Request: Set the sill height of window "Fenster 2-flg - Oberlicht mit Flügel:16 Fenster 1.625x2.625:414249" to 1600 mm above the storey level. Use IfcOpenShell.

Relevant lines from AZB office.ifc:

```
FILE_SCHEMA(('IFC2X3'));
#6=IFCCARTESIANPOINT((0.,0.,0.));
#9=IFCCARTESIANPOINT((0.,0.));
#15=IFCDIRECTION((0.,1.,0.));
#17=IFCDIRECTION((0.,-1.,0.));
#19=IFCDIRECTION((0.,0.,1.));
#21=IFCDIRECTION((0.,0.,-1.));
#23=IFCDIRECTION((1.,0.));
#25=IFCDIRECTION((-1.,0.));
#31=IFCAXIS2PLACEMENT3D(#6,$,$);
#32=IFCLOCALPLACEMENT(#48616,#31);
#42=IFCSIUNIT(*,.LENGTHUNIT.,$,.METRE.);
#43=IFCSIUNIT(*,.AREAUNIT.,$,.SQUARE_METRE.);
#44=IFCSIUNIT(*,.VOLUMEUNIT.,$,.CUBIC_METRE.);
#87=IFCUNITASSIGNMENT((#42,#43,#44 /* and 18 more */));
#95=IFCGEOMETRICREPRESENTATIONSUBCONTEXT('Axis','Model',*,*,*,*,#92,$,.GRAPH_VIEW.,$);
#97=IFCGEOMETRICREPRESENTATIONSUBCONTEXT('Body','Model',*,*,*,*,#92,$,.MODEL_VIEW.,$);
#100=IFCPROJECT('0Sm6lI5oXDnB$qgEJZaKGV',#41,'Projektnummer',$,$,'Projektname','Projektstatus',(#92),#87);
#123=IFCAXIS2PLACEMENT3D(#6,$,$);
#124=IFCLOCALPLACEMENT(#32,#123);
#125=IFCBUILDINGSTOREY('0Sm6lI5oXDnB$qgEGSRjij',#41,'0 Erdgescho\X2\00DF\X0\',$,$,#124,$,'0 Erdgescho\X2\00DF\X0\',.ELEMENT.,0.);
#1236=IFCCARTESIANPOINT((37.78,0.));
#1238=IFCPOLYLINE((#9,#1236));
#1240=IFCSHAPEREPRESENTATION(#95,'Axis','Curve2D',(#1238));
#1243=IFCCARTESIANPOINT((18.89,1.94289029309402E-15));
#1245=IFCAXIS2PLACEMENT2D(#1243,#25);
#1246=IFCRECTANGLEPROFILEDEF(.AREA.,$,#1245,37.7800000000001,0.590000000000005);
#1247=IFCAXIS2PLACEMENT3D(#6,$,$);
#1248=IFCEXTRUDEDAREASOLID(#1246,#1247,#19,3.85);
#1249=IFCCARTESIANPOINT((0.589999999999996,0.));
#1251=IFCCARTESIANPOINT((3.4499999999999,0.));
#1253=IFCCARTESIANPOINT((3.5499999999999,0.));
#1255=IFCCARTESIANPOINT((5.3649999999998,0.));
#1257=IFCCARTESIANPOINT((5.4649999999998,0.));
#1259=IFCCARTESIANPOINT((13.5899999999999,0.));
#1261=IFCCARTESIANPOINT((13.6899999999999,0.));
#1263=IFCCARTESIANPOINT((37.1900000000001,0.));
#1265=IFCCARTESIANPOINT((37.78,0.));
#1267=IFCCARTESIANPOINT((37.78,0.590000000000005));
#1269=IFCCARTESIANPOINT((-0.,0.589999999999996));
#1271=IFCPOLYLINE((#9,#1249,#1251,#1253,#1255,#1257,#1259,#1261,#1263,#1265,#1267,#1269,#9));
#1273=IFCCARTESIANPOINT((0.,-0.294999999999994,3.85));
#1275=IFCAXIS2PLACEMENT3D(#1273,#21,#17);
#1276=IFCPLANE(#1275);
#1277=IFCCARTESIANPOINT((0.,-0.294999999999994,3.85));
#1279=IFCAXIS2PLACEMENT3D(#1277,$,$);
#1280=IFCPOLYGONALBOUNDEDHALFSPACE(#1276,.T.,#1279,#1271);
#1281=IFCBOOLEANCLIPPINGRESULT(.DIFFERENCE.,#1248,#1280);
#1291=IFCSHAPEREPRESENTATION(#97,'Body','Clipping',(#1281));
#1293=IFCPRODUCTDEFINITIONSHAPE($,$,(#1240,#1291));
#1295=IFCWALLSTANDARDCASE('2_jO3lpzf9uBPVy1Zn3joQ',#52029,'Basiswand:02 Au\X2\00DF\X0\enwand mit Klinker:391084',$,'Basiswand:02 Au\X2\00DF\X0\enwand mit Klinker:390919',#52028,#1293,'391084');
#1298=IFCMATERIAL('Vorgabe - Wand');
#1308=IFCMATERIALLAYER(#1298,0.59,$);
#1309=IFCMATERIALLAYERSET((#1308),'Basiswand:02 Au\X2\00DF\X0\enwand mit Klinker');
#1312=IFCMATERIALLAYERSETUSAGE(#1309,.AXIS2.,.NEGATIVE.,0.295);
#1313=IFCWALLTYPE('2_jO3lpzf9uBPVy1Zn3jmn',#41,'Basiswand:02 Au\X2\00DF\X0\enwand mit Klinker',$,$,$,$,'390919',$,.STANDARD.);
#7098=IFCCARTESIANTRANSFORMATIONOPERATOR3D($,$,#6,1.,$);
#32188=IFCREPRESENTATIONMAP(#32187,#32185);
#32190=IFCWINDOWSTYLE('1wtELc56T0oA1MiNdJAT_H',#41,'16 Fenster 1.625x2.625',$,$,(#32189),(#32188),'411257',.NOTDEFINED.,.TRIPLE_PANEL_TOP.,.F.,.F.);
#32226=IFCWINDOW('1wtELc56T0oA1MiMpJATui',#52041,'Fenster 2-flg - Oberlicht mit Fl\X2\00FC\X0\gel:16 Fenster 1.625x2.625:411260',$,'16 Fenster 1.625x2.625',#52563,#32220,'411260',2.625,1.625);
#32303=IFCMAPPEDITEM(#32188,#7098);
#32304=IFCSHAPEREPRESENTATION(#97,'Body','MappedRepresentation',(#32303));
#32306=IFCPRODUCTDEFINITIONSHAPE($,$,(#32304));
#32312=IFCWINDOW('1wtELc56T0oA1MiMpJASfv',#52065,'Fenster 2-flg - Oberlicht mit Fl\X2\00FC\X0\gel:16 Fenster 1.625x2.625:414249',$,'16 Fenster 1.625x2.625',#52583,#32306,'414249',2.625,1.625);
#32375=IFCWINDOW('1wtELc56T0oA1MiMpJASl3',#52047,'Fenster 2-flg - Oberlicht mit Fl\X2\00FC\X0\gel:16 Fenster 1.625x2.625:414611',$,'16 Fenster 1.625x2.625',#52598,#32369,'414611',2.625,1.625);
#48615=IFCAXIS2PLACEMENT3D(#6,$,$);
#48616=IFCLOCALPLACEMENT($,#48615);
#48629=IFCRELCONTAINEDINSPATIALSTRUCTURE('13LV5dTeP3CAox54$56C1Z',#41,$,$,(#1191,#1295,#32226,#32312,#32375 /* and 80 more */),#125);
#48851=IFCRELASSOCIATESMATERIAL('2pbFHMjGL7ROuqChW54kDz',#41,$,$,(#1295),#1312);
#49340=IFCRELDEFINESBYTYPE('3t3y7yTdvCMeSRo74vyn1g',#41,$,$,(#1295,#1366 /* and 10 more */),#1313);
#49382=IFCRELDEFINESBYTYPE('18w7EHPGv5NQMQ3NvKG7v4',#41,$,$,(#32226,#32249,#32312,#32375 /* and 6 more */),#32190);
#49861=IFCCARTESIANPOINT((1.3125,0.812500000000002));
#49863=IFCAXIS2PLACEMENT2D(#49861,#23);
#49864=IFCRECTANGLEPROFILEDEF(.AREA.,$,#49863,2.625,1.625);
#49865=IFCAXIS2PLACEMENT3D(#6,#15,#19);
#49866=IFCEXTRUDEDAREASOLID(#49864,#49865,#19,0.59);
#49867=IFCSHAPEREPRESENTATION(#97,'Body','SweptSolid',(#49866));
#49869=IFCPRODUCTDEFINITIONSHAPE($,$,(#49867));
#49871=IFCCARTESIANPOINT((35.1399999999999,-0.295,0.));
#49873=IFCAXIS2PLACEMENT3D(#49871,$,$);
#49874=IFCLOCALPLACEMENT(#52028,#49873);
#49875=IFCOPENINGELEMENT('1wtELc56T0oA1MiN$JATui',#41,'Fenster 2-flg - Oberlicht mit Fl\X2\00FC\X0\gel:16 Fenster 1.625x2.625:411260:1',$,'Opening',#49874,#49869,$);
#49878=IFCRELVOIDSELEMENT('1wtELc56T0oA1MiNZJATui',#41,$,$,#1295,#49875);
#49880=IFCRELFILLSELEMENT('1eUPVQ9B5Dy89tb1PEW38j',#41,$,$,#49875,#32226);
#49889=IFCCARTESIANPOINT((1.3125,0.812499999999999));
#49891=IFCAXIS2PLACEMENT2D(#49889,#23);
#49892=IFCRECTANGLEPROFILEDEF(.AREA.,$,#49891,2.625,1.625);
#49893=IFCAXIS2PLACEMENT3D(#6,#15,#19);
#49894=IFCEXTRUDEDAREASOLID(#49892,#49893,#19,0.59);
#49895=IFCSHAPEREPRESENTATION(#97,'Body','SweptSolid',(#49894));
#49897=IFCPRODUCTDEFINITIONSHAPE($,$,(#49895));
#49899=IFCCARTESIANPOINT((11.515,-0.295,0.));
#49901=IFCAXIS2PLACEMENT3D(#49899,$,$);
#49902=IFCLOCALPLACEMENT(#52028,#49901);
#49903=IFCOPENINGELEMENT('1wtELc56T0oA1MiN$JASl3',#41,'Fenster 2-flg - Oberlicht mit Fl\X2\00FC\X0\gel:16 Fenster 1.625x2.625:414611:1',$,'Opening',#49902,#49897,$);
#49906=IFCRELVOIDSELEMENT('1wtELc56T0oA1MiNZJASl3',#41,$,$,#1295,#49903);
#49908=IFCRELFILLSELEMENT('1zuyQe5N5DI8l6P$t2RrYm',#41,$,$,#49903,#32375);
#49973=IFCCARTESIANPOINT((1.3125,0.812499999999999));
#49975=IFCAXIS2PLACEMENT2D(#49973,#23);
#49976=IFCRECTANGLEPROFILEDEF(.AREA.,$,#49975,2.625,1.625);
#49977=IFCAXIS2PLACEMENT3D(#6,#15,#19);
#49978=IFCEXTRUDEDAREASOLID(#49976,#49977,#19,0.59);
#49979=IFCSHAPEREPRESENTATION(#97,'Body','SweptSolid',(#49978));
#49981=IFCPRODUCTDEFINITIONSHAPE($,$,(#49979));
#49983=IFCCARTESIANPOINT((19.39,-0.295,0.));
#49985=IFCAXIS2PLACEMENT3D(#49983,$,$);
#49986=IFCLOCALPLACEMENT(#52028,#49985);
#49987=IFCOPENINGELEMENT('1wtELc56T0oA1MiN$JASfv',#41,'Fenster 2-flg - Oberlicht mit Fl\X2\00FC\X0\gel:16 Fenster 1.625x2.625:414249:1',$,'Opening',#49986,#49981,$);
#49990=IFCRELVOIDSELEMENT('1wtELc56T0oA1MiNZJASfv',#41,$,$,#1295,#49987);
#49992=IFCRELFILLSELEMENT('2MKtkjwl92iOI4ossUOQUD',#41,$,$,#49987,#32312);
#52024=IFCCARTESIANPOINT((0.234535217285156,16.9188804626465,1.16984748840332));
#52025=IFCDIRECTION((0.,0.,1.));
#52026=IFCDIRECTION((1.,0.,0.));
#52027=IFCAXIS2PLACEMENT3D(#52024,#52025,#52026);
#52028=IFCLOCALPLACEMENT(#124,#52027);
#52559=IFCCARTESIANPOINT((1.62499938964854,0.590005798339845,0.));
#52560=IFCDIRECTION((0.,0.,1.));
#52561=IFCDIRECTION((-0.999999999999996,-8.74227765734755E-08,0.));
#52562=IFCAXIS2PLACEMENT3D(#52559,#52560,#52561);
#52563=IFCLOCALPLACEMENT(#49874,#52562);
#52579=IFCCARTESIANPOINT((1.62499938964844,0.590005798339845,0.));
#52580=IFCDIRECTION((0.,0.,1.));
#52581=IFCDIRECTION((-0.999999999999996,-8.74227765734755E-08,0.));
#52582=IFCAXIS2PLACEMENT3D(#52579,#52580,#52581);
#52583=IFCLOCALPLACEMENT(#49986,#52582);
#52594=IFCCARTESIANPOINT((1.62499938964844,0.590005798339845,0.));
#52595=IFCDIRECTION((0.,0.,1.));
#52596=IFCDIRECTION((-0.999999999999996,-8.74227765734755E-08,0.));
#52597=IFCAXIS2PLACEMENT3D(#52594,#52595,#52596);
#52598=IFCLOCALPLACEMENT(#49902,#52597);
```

```python
import numpy as np
import ifcopenshell
import ifcopenshell.api.geometry
import ifcopenshell.geom
import ifcopenshell.util.element
import ifcopenshell.util.placement
import ifcopenshell.util.shape
import ifcopenshell.util.unit

model = ifcopenshell.open("AZB office.ifc")
unit_scale = ifcopenshell.util.unit.calculate_unit_scale(model)

window = model.by_guid("1wtELc56T0oA1MiMpJASfv")
opening = window.FillsVoids[0].RelatingOpeningElement
storey = ifcopenshell.util.element.get_container(window, ifc_class="IfcBuildingStorey")
level = ifcopenshell.util.placement.get_local_placement(storey.ObjectPlacement)[2, 3]

# The opening's origin need not be at the sill, so measure its lowest point.
shape = ifcopenshell.geom.create_shape(ifcopenshell.geom.settings(), opening)
bottom = ifcopenshell.util.shape.get_shape_bottom_elevation(shape, shape.geometry) / unit_scale
dz = level + 1.6 / unit_scale - bottom

shift = np.array([0.0, 0.0, dz])
# The window is placed relative to its opening, so it follows when the opening moves.
matrix = ifcopenshell.util.placement.get_local_placement(opening.ObjectPlacement)
matrix[:3, 3] += shift
ifcopenshell.api.geometry.edit_object_placement(
    model, product=opening, matrix=matrix, is_si=False, should_transform_children=True
)

print(f"moved by {dz * unit_scale:+.3f} m")

model.write("AZB office_v2.ifc")
```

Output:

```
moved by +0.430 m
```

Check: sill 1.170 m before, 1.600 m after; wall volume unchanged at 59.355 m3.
